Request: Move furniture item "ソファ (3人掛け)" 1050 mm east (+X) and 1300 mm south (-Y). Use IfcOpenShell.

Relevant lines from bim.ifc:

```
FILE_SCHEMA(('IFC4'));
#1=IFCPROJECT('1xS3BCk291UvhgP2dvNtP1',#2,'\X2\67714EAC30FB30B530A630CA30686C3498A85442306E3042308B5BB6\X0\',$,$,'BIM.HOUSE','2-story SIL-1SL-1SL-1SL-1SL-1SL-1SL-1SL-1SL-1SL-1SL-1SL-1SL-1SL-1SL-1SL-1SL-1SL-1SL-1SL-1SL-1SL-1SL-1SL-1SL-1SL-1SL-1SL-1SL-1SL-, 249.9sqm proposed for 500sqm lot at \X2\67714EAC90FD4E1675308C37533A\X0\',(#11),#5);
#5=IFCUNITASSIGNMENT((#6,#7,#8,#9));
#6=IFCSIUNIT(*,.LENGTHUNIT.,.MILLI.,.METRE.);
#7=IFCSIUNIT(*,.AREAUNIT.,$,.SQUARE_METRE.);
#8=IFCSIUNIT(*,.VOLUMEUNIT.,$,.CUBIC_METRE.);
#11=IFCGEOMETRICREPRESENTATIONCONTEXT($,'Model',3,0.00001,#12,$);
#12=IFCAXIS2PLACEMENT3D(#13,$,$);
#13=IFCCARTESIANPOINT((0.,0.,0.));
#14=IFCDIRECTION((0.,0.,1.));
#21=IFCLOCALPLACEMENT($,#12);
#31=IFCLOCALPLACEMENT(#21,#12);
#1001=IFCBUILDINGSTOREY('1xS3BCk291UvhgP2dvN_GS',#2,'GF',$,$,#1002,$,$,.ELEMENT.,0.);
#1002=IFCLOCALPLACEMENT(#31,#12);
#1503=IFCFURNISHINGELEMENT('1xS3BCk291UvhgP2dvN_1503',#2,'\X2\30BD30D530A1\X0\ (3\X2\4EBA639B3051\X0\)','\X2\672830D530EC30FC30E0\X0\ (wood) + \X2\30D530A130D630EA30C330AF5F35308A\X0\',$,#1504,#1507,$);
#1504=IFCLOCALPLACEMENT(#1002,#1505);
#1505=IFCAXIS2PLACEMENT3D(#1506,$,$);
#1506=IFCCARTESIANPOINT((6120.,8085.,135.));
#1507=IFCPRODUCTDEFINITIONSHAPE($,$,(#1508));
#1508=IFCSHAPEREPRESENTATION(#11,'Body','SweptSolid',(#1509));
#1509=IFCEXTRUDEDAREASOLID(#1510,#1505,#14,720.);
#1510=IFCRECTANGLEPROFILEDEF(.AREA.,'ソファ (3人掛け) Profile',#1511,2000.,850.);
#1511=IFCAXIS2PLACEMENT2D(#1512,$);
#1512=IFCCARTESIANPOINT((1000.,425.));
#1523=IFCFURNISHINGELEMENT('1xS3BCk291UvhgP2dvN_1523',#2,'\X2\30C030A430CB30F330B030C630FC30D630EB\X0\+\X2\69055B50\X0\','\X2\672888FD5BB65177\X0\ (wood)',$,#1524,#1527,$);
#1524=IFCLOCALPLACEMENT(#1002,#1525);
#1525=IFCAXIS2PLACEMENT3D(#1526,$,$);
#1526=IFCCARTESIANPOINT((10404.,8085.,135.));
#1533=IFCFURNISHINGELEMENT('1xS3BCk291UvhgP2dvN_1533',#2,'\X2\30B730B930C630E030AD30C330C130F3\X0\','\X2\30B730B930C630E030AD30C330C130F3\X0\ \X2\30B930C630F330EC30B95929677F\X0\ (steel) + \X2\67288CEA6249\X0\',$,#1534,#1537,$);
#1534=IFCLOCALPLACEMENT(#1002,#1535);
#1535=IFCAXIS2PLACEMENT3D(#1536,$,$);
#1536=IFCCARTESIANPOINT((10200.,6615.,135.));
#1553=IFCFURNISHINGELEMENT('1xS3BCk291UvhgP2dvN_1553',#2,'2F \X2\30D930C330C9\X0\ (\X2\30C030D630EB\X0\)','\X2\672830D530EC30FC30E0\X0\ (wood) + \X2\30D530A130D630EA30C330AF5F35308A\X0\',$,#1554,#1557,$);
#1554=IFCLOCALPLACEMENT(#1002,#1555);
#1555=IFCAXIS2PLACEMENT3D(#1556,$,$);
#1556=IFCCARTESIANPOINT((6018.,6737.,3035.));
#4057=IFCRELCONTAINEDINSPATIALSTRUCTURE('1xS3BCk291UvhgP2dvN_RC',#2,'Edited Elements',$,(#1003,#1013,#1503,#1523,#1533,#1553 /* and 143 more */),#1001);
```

```python
import ifcopenshell
import ifcopenshell.api.geometry
import ifcopenshell.util.placement

model = ifcopenshell.open("bim.ifc")

item = model.by_id(1503)
matrix = ifcopenshell.util.placement.get_local_placement(item.ObjectPlacement)
matrix[0, 3] += 1050.0
matrix[1, 3] -= 1300.0
ifcopenshell.api.geometry.edit_object_placement(model, product=item, matrix=matrix, is_si=False)

print(ifcopenshell.util.placement.get_local_placement(item.ObjectPlacement).round(3) + 0.0)

model.write("bim-out.ifc")
```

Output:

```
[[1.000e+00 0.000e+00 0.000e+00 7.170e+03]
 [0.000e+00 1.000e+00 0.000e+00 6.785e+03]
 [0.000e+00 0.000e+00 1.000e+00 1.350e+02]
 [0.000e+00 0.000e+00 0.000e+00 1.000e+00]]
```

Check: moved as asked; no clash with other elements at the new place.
